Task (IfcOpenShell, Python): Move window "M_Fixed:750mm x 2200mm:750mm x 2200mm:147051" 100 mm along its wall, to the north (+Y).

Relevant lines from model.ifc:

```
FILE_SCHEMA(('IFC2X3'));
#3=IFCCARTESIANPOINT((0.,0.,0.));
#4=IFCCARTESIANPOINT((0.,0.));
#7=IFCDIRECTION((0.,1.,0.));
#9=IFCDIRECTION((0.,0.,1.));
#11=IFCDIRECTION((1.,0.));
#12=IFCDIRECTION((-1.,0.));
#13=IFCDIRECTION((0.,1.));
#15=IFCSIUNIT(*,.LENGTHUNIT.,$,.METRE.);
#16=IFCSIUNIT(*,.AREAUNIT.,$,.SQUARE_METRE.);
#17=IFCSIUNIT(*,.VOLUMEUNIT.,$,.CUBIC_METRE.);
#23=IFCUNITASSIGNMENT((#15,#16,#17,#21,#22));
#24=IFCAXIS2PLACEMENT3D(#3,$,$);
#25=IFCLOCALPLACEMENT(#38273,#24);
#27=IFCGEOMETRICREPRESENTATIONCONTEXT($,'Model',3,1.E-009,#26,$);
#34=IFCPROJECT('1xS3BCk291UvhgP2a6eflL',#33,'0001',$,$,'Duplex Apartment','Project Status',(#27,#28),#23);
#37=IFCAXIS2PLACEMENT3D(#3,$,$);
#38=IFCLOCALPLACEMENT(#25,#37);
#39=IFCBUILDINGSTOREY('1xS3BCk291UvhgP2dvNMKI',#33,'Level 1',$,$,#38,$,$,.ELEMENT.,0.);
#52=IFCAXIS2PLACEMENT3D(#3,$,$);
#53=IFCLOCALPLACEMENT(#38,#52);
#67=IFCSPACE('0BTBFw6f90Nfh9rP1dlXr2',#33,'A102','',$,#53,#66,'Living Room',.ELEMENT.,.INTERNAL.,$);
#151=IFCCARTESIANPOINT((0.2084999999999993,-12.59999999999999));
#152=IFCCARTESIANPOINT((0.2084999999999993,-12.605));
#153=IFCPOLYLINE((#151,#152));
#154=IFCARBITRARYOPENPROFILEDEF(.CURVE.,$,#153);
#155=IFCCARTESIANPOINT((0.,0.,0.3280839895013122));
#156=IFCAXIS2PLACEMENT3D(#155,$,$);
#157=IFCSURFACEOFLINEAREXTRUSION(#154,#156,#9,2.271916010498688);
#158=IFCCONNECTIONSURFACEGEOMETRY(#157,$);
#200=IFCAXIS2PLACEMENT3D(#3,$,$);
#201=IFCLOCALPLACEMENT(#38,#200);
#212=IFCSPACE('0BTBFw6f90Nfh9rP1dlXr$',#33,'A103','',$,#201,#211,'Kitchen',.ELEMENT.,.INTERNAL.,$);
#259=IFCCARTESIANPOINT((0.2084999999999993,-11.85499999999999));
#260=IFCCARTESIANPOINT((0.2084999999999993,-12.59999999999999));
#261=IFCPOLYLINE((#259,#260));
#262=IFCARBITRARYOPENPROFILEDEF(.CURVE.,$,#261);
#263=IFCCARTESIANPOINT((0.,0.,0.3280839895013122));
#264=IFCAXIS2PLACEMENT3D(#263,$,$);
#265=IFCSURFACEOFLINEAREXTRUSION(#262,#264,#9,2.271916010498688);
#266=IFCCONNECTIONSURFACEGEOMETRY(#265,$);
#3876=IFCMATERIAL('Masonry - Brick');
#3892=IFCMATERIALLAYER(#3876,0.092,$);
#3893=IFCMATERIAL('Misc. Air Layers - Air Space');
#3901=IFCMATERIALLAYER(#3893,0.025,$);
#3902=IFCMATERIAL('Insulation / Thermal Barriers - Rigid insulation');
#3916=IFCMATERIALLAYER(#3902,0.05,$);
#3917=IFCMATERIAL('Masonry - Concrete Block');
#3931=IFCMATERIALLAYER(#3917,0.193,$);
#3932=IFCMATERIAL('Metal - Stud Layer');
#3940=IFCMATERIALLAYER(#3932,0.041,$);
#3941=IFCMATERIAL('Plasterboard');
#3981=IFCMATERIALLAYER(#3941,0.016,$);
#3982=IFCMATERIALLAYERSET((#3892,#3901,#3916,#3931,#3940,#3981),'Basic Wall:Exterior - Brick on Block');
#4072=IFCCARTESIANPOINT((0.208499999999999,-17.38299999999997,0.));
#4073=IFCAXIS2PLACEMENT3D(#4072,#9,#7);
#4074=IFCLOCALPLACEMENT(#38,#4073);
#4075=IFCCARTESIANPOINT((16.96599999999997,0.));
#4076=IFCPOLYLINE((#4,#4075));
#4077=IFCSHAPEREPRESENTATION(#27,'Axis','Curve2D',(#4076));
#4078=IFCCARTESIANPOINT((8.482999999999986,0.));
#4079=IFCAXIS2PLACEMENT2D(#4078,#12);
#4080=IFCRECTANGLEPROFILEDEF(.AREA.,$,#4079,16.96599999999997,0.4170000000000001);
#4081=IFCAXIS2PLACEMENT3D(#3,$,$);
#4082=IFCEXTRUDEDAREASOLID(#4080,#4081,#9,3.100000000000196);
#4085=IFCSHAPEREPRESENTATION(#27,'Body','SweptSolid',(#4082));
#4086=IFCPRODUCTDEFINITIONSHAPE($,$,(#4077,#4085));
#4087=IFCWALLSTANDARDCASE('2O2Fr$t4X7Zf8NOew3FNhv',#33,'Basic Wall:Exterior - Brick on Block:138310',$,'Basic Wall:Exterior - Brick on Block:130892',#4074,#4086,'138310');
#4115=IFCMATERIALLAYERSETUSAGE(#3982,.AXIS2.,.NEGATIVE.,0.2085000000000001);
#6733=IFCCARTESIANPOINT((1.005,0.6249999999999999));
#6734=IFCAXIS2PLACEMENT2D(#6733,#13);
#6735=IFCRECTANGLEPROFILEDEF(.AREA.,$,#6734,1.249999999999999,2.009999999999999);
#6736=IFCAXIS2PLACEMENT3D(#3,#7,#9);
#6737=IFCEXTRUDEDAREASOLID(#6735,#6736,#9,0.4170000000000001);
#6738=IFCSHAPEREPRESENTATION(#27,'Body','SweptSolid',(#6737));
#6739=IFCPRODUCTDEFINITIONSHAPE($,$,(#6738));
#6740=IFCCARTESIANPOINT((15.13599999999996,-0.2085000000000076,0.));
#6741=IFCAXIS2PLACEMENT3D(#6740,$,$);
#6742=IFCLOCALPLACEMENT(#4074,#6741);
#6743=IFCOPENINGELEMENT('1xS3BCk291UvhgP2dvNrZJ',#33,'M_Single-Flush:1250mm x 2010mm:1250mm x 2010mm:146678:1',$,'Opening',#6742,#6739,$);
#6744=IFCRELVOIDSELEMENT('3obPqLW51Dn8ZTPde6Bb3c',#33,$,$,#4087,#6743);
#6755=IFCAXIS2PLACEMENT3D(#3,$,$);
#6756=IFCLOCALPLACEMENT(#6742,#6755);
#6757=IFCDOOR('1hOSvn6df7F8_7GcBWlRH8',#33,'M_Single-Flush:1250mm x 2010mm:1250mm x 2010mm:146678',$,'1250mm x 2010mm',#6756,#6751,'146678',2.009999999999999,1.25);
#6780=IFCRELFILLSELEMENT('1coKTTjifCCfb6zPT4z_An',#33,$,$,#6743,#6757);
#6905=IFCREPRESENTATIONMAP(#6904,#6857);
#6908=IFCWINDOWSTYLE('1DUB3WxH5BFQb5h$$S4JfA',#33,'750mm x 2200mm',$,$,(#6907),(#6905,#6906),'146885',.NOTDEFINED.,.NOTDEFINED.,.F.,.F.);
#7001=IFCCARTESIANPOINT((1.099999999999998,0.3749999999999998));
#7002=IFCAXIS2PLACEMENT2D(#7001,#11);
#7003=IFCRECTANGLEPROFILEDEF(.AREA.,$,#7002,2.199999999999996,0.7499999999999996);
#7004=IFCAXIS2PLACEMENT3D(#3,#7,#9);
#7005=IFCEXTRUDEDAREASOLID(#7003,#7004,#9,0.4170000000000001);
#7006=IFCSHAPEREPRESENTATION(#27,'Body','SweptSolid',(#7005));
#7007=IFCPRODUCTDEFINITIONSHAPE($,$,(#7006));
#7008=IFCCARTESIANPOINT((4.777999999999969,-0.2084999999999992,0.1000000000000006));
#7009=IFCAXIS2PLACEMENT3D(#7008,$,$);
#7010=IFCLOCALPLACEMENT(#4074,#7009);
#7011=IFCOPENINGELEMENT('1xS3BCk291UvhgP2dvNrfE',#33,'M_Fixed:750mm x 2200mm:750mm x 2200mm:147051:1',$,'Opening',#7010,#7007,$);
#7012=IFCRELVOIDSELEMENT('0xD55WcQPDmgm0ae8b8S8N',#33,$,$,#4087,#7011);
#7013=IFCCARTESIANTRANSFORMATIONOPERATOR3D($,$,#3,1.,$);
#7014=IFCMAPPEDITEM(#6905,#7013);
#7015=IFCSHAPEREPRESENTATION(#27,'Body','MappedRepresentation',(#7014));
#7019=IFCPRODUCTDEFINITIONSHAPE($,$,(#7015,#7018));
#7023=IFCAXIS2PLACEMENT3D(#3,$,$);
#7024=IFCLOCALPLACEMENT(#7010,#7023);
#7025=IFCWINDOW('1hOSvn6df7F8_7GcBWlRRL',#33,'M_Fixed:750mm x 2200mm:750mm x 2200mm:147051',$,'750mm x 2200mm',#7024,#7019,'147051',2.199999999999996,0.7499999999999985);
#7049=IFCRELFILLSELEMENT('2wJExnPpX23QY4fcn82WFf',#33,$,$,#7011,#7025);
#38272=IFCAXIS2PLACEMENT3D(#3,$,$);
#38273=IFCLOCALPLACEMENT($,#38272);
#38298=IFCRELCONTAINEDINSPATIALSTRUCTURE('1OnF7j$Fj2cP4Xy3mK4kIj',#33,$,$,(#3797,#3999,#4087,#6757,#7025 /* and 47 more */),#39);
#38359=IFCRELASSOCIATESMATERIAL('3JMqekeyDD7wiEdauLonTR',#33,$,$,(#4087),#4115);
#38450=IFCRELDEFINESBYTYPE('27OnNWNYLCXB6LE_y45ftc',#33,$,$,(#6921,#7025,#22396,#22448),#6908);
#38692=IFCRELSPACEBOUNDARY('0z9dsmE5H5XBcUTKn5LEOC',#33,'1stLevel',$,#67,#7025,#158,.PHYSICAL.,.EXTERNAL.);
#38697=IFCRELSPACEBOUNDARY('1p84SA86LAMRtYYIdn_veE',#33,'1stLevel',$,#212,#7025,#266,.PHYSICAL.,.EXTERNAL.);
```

```python
import numpy as np
import ifcopenshell
import ifcopenshell.api.geometry
import ifcopenshell.util.placement

model = ifcopenshell.open("model.ifc")

window = model.by_id(7025)
opening = window.FillsVoids[0].RelatingOpeningElement
wall = opening.VoidsElements[0].RelatingBuildingElement

wall_matrix = ifcopenshell.util.placement.get_local_placement(wall.ObjectPlacement)
shift = wall_matrix[:3, 0] * 0.1
before = ifcopenshell.util.placement.get_local_placement(window.ObjectPlacement)[:3, 3].copy()

# The window is placed relative to its opening, so it follows when the opening moves.
matrix = ifcopenshell.util.placement.get_local_placement(opening.ObjectPlacement)
matrix[:3, 3] += shift
ifcopenshell.api.geometry.edit_object_placement(
    model, product=opening, matrix=matrix, is_si=False, should_transform_children=True
)

# Space boundary surfaces are stored in each space's coordinates; move them too.
for rel in window.ProvidesBoundaries:
    if not rel.ConnectionGeometry:
        continue
    surface = rel.ConnectionGeometry.SurfaceOnRelatingElement
    space_matrix = ifcopenshell.util.placement.get_local_placement(rel.RelatingSpace.ObjectPlacement)
    point = np.array(surface.Position.Location.Coordinates) + space_matrix[:3, :3].T @ shift
    surface.Position = model.createIfcAxis2Placement3D(
        model.createIfcCartesianPoint(point.tolist()), surface.Position.Axis, surface.Position.RefDirection
    )

after = ifcopenshell.util.placement.get_local_placement(window.ObjectPlacement)[:3, 3]
print("window moved by", (after - before).round(3) + 0.0)

model.write("model_v2.ifc")
```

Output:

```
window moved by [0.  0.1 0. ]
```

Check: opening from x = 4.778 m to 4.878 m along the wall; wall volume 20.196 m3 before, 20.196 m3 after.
